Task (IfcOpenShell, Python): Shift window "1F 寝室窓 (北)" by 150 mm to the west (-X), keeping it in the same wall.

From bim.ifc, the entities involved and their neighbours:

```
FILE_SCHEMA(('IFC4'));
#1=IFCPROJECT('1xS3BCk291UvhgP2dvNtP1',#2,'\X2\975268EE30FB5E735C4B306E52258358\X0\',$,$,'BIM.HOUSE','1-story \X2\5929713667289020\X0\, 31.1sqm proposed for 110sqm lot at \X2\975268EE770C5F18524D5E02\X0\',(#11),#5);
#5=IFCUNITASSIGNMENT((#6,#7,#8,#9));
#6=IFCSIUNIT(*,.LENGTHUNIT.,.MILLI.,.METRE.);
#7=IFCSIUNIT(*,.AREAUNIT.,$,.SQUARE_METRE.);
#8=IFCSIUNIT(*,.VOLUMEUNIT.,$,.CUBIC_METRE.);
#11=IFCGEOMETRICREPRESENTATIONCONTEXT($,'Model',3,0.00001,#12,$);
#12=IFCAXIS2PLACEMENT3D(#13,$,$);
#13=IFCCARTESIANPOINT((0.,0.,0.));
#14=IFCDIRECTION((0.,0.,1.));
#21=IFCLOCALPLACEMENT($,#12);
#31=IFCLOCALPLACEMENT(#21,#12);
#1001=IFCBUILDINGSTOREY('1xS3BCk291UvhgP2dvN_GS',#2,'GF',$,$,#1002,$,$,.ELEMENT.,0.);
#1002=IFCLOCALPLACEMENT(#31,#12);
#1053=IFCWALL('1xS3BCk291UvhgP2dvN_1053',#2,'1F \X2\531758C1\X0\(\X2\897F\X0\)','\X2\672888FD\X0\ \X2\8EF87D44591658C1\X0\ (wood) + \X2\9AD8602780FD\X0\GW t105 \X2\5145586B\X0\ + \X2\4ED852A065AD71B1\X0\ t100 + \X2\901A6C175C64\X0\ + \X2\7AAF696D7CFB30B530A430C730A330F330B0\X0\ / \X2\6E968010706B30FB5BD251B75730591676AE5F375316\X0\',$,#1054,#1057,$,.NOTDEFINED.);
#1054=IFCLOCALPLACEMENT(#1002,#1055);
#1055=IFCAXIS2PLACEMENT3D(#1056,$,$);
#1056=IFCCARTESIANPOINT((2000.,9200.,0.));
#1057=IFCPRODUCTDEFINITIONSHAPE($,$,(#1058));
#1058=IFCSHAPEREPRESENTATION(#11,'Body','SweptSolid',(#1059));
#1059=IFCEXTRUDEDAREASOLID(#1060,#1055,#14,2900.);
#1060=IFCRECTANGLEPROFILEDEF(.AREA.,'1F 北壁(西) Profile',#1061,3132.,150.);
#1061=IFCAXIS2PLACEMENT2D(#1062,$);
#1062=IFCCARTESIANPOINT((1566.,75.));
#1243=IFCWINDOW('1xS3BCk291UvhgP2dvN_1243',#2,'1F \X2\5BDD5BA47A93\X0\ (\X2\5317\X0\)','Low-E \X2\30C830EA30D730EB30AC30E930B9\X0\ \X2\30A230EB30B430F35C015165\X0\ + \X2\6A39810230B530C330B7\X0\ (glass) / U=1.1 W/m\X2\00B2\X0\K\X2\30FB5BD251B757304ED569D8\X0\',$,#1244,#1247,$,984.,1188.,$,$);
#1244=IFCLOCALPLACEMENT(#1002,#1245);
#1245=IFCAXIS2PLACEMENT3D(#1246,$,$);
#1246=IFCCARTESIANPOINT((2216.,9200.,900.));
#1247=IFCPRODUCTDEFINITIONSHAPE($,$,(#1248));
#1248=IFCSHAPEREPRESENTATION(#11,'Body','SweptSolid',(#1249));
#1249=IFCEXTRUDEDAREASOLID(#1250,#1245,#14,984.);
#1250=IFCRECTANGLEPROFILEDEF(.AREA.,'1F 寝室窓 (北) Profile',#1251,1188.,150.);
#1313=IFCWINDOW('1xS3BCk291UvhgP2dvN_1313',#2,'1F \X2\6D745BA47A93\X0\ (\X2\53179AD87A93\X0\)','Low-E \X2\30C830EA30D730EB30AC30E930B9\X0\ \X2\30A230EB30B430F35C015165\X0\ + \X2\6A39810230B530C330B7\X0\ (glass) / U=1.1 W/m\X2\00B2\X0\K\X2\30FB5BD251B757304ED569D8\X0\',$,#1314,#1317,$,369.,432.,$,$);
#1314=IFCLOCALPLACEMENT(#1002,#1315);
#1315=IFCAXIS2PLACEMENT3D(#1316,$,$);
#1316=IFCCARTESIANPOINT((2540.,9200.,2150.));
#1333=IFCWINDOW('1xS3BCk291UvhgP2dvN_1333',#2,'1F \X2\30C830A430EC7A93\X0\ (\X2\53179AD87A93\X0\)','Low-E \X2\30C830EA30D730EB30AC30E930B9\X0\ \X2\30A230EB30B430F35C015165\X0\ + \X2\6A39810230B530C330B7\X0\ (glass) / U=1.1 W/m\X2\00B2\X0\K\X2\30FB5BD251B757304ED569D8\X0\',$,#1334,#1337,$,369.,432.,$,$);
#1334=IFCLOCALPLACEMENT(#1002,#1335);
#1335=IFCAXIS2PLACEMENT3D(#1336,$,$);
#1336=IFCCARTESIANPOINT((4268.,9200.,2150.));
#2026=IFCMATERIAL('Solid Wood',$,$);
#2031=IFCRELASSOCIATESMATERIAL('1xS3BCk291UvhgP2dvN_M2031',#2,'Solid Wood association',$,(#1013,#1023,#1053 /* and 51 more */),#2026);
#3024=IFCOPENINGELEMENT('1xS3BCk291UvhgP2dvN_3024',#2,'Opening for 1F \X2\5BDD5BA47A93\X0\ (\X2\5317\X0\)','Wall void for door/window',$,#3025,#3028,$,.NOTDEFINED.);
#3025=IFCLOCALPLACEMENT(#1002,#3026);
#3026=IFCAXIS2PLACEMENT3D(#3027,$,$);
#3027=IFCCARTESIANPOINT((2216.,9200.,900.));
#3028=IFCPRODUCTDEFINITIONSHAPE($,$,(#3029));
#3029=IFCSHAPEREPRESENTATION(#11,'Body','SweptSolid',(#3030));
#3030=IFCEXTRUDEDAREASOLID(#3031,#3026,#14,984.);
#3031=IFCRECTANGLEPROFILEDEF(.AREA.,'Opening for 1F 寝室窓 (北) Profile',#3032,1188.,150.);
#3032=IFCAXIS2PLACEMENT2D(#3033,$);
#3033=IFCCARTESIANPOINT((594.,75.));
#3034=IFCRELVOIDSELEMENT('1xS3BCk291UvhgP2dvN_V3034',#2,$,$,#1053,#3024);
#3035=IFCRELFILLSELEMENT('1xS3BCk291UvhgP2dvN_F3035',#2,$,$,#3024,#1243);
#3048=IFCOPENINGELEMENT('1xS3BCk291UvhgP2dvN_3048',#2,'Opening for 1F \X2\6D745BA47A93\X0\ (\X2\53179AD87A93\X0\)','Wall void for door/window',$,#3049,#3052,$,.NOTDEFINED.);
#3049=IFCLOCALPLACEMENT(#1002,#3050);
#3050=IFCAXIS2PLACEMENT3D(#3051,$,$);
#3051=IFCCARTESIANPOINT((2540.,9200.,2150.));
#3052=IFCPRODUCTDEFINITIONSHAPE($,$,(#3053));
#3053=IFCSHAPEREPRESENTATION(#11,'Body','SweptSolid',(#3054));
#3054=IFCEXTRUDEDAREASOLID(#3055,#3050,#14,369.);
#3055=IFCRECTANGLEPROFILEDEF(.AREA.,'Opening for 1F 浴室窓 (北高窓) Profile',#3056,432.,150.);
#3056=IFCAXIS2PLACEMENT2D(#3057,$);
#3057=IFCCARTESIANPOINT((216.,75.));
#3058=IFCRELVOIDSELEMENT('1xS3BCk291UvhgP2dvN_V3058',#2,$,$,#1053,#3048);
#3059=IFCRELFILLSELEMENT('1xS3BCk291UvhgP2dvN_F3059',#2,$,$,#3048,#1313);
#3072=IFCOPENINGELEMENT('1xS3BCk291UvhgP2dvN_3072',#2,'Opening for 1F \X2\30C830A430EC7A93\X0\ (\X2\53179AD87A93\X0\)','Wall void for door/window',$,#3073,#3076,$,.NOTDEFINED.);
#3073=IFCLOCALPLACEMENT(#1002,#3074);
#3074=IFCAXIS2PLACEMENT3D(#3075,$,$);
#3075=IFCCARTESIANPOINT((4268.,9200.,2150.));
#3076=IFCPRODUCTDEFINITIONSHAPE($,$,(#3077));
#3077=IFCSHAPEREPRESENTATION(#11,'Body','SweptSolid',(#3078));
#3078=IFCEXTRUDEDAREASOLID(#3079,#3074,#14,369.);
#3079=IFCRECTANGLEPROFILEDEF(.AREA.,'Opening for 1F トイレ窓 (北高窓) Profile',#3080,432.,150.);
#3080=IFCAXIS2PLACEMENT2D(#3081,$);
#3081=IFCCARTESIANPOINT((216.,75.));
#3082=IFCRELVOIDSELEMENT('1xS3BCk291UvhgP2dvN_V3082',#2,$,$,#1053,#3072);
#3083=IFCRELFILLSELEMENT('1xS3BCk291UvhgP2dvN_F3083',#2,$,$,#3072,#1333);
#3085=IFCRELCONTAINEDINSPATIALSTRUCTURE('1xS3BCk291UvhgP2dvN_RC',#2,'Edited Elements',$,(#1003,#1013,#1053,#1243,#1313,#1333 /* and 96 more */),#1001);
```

```python
import ifcopenshell
import ifcopenshell.api.geometry
import ifcopenshell.util.placement
import ifcopenshell.util.unit

model = ifcopenshell.open("bim.ifc")
unit_scale = ifcopenshell.util.unit.calculate_unit_scale(model)

window = model.by_id(1243)
opening = window.FillsVoids[0].RelatingOpeningElement
wall = opening.VoidsElements[0].RelatingBuildingElement

wall_matrix = ifcopenshell.util.placement.get_local_placement(wall.ObjectPlacement)
shift = wall_matrix[:3, 0] * -0.15 / unit_scale
before = ifcopenshell.util.placement.get_local_placement(window.ObjectPlacement)[:3, 3].copy()

# The window is not placed relative to its opening, so move both.
for product in (opening, window):
    matrix = ifcopenshell.util.placement.get_local_placement(product.ObjectPlacement)
    matrix[:3, 3] += shift
    ifcopenshell.api.geometry.edit_object_placement(model, product=product, matrix=matrix, is_si=False)

after = ifcopenshell.util.placement.get_local_placement(window.ObjectPlacement)[:3, 3]
print("window moved by", (after - before).round(3) + 0.0)

model.write("bim_updated.ifc")
```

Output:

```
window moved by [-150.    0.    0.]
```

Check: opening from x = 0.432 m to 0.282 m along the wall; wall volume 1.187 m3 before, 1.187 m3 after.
